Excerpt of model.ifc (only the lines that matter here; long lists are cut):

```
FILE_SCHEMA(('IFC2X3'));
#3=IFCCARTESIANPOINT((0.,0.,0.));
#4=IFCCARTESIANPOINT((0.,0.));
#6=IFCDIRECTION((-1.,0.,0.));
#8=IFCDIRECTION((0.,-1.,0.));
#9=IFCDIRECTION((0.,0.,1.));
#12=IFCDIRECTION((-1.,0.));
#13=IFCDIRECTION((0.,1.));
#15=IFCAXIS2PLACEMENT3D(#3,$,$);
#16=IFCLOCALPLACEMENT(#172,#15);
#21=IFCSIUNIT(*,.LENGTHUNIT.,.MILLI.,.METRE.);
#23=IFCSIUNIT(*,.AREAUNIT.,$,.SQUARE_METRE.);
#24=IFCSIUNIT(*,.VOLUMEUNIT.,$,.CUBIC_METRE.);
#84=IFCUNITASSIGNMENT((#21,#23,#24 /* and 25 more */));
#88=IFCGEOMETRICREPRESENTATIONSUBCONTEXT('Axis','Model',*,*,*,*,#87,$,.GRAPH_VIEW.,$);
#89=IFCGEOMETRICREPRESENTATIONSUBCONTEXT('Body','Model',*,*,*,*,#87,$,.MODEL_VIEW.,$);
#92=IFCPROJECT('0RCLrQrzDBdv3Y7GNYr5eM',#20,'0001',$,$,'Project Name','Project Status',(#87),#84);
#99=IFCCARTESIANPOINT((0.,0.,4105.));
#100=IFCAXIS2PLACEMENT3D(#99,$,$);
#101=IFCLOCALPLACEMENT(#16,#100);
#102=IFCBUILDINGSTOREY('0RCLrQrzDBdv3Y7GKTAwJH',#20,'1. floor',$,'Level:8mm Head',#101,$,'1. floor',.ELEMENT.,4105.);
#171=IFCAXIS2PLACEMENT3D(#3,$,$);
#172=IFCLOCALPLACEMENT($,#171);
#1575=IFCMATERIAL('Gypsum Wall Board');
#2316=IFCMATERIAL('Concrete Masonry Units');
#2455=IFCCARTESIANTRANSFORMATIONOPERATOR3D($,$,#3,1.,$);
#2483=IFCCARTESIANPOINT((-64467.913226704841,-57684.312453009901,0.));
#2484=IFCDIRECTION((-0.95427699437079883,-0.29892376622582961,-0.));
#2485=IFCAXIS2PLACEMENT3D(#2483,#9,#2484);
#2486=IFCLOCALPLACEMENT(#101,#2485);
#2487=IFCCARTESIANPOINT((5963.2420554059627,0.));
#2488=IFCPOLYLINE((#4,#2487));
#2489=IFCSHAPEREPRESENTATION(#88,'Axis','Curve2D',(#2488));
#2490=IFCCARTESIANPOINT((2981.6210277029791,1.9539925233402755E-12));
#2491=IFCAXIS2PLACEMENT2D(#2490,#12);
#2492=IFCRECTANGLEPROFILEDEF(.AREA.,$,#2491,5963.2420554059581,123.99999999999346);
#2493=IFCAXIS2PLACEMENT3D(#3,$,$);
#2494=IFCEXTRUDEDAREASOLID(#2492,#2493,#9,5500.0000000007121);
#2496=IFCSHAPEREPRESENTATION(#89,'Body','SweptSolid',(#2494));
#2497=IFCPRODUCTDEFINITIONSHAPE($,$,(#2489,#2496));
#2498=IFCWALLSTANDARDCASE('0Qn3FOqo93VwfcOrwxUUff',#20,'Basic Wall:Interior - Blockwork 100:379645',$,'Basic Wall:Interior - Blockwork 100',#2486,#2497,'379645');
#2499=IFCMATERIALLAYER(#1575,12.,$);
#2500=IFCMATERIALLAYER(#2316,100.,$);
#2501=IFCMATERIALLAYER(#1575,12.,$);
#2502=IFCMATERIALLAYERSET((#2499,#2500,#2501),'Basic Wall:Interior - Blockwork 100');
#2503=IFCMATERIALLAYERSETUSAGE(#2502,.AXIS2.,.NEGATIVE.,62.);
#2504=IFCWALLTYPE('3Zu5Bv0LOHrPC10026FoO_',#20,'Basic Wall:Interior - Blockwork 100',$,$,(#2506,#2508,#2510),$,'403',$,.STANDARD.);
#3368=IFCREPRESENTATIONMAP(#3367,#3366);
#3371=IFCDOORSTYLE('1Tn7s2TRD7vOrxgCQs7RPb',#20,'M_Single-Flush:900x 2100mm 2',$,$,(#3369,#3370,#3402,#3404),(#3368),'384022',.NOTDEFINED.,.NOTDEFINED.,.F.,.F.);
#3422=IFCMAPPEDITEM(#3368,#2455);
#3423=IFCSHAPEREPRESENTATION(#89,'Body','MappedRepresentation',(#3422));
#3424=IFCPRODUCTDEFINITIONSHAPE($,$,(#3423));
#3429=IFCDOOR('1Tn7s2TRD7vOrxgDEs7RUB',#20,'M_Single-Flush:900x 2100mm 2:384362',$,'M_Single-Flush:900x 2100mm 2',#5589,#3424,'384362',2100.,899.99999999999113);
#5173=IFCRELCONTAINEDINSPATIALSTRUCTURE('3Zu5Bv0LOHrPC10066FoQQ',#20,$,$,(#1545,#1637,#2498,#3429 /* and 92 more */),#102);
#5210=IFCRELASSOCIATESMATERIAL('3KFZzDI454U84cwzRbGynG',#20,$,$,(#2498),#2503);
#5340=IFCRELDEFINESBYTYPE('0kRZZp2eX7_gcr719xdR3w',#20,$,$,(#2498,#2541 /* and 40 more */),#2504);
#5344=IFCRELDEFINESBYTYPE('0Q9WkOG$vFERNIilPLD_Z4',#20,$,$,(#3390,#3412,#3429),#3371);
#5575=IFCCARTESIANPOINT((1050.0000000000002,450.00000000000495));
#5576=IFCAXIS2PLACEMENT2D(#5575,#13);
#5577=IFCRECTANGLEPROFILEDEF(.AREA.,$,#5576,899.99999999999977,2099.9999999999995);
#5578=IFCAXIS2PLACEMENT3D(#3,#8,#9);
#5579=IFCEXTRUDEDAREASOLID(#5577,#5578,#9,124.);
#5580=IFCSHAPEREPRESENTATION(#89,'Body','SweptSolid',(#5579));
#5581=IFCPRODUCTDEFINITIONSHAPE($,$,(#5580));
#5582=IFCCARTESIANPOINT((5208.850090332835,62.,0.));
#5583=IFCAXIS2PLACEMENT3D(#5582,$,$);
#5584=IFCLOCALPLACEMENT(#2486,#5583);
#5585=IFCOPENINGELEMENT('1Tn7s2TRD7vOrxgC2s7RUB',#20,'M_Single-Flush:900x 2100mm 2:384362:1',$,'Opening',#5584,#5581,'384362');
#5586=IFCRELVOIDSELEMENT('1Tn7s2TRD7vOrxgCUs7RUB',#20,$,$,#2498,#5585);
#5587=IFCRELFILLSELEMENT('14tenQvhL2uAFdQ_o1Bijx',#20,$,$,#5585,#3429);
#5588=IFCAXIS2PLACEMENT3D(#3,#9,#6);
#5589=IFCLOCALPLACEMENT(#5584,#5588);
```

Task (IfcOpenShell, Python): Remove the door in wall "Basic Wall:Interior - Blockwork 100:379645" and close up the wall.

```python
import ifcopenshell
import ifcopenshell.api.feature
import ifcopenshell.api.root
import ifcopenshell.geom
import ifcopenshell.util.shape

model = ifcopenshell.open("model.ifc")
settings = ifcopenshell.geom.settings()


def volume(element):
    """Net volume in cubic metres, openings subtracted."""
    shape = ifcopenshell.geom.create_shape(settings, element)
    return ifcopenshell.util.shape.get_volume(shape.geometry)


door = model.by_id(3429)
opening = door.FillsVoids[0].RelatingOpeningElement
wall = opening.VoidsElements[0].RelatingBuildingElement
before = volume(wall)

ifcopenshell.api.root.remove_product(model, product=door)
ifcopenshell.api.feature.remove_feature(model, feature=opening)

after = volume(wall)

print(f"wall volume {before:.3f} -> {after:.3f} m3")

model.write("model_updated.ifc")
```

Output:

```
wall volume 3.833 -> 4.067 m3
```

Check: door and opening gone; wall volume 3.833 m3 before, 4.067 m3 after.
